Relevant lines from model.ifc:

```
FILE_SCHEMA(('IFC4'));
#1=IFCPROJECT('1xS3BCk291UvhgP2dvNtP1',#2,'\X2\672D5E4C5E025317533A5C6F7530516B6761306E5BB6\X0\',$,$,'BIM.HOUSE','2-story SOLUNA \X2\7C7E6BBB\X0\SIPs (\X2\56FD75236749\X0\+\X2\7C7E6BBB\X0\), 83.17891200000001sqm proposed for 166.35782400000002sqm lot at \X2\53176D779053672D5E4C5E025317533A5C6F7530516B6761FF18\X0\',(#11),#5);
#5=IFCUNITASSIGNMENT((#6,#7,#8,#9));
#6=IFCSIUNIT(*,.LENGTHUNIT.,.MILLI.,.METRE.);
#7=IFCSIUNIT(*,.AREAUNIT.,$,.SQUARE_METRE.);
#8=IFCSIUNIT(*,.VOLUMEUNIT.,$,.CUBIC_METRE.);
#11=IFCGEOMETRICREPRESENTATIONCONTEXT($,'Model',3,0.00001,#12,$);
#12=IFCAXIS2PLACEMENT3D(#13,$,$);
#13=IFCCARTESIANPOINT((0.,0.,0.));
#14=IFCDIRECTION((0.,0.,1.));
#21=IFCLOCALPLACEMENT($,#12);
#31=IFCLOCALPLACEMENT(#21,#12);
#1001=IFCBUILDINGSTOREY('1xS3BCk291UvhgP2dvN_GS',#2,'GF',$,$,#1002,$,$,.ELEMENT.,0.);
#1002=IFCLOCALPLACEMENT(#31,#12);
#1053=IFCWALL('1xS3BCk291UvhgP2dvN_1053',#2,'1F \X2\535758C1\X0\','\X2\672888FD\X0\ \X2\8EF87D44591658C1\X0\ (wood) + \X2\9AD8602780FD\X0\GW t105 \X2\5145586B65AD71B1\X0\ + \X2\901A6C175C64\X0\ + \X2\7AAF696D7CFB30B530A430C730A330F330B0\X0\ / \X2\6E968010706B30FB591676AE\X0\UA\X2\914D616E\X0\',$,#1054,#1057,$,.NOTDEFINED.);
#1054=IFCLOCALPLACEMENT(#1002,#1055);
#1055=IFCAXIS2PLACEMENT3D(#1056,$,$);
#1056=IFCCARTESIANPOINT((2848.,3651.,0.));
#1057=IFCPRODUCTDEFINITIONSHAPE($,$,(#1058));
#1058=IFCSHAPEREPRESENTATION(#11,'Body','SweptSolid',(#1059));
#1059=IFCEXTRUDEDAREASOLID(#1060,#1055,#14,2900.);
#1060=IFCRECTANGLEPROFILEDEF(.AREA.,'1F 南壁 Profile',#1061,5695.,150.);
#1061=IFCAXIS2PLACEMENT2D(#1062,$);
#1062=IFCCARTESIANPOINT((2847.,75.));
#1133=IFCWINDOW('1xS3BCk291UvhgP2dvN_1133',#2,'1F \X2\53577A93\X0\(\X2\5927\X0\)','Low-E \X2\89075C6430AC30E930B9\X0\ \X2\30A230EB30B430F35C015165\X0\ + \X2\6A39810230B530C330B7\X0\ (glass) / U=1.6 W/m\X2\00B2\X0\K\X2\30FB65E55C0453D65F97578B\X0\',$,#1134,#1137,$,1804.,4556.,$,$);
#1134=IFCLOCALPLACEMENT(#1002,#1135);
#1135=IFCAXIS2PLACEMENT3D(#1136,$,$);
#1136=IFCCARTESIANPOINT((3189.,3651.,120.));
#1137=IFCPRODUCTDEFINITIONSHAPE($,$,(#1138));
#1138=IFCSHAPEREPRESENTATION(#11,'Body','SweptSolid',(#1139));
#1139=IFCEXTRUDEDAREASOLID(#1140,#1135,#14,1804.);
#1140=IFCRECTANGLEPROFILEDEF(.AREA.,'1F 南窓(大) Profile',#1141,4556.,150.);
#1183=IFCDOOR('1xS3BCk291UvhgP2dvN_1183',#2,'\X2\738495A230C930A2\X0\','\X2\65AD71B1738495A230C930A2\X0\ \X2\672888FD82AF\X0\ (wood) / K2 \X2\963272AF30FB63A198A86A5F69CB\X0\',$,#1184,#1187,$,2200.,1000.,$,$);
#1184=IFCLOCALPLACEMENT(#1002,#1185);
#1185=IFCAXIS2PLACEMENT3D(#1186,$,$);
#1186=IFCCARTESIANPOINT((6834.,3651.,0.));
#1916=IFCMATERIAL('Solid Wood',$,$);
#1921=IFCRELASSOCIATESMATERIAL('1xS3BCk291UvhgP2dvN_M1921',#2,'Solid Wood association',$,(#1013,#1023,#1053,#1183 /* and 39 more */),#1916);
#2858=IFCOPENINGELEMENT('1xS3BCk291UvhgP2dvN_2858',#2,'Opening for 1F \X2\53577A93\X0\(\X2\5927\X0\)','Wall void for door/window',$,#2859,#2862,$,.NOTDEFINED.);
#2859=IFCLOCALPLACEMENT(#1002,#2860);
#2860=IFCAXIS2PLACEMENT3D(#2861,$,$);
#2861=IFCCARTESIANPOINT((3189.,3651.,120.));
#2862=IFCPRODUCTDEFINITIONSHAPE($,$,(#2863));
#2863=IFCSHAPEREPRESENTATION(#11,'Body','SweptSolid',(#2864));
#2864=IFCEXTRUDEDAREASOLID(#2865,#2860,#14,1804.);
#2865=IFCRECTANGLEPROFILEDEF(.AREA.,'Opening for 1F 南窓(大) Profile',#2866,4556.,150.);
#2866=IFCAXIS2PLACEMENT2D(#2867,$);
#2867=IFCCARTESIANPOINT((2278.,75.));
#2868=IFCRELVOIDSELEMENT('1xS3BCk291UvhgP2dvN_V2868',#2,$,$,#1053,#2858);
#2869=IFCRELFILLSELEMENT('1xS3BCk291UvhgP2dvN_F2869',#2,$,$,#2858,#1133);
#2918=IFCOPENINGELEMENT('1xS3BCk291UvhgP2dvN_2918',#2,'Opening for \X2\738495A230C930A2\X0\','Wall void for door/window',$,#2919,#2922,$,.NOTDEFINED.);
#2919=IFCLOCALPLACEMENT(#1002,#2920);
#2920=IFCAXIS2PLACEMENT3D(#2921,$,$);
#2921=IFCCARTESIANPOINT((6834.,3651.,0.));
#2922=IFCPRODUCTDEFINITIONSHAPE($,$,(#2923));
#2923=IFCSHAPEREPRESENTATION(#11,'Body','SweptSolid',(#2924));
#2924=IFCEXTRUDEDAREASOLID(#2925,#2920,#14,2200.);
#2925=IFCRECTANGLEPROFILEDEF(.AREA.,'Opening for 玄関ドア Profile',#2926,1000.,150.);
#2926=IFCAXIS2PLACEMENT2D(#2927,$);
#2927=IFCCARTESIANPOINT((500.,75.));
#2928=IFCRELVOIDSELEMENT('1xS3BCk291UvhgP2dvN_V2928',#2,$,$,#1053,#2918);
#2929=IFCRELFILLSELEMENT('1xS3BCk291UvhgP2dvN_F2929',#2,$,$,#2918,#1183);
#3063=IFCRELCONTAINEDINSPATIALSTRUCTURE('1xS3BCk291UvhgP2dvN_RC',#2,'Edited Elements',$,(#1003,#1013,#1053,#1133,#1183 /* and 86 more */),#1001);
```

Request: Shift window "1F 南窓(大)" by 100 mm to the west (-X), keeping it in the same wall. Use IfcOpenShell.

```python
import ifcopenshell
import ifcopenshell.api.geometry
import ifcopenshell.util.placement

model = ifcopenshell.open("model.ifc")

window = model.by_guid("1xS3BCk291UvhgP2dvN_1133")
opening = window.FillsVoids[0].RelatingOpeningElement
wall = opening.VoidsElements[0].RelatingBuildingElement

wall_matrix = ifcopenshell.util.placement.get_local_placement(wall.ObjectPlacement)
shift = wall_matrix[:3, 0] * -100.0
before = ifcopenshell.util.placement.get_local_placement(window.ObjectPlacement)[:3, 3].copy()

# The window is not placed relative to its opening, so move both.
for product in (opening, window):
    matrix = ifcopenshell.util.placement.get_local_placement(product.ObjectPlacement)
    matrix[:3, 3] += shift
    ifcopenshell.api.geometry.edit_object_placement(model, product=product, matrix=matrix, is_si=False)

after = ifcopenshell.util.placement.get_local_placement(window.ObjectPlacement)[:3, 3]
print("window moved by", (after - before).round(3) + 0.0)

model.write("model_updated.ifc")
```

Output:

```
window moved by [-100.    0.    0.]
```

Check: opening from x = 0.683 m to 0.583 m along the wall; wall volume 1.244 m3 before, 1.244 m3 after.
